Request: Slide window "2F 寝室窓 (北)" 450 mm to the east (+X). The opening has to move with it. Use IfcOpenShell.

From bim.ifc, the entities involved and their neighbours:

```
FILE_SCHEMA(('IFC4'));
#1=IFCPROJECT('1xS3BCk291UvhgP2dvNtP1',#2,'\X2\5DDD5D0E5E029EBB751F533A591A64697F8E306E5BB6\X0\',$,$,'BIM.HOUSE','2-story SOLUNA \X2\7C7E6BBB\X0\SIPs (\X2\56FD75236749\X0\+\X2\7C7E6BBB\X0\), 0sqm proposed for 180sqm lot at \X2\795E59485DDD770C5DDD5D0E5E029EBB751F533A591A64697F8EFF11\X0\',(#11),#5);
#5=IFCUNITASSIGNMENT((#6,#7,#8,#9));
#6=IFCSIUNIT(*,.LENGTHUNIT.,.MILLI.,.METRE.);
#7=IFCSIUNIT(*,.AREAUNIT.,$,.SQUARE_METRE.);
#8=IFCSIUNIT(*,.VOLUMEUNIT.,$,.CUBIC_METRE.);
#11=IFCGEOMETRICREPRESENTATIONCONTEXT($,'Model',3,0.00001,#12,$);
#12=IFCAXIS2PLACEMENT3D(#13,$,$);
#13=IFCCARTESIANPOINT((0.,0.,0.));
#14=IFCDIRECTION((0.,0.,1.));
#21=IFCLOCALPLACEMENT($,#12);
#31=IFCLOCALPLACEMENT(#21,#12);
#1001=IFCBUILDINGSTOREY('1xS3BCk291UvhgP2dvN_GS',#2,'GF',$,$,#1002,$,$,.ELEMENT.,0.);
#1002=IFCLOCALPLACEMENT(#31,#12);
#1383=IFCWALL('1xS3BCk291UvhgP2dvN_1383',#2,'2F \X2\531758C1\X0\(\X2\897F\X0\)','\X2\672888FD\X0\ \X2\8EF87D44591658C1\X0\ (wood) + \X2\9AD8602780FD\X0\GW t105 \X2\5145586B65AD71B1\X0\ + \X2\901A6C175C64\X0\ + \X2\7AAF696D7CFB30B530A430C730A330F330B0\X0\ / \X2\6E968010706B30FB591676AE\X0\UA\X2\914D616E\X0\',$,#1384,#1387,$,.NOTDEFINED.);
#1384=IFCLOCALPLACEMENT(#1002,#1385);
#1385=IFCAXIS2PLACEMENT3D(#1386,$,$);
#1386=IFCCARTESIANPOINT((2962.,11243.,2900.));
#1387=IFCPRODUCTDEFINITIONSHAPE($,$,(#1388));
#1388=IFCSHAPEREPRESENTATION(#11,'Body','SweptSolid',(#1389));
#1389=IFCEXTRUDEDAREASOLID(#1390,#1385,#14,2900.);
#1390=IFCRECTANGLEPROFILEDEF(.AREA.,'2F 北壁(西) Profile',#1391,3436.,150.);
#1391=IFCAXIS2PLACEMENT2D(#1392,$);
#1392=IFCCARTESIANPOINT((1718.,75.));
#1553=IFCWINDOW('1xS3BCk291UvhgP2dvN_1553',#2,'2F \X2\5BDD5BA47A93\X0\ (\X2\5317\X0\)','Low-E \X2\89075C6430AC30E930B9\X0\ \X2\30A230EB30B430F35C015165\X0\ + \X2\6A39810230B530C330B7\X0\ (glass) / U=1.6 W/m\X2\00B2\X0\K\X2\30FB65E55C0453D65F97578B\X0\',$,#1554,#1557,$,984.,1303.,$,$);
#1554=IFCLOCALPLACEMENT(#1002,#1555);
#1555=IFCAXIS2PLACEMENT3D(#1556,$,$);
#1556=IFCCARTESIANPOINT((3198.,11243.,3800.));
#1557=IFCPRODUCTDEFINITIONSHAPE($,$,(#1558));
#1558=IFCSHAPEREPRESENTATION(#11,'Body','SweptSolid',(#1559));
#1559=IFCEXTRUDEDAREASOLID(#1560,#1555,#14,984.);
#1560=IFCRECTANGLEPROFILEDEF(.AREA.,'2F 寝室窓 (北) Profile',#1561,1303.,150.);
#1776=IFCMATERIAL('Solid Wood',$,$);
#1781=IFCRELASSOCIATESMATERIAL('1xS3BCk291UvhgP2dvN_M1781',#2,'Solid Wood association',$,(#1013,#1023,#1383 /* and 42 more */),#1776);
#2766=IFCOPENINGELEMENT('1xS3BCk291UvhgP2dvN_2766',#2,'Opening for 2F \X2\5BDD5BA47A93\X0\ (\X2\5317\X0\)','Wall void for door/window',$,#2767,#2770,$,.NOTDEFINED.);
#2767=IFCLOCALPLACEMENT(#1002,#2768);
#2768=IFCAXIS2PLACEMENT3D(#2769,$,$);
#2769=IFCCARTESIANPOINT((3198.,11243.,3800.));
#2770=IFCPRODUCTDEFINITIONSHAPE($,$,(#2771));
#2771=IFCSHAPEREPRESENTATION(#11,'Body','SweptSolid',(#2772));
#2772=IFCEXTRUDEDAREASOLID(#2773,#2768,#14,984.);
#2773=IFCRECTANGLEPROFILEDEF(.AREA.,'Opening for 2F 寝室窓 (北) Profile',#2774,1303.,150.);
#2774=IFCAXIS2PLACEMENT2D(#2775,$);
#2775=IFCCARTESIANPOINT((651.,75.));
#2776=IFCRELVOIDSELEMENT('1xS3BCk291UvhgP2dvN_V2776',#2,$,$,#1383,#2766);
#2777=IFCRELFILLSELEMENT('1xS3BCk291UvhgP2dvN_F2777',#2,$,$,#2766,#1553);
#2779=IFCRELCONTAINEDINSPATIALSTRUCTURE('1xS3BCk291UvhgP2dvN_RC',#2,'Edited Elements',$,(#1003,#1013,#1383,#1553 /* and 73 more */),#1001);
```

```python
import ifcopenshell
import ifcopenshell.api.geometry
import ifcopenshell.util.placement
import ifcopenshell.util.unit

model = ifcopenshell.open("bim.ifc")
unit_scale = ifcopenshell.util.unit.calculate_unit_scale(model)

window = model.by_guid("1xS3BCk291UvhgP2dvN_1553")
opening = window.FillsVoids[0].RelatingOpeningElement
wall = opening.VoidsElements[0].RelatingBuildingElement

wall_matrix = ifcopenshell.util.placement.get_local_placement(wall.ObjectPlacement)
shift = wall_matrix[:3, 0] * 0.45 / unit_scale
before = ifcopenshell.util.placement.get_local_placement(window.ObjectPlacement)[:3, 3].copy()

# The window is not placed relative to its opening, so move both.
for product in (opening, window):
    matrix = ifcopenshell.util.placement.get_local_placement(product.ObjectPlacement)
    matrix[:3, 3] += shift
    ifcopenshell.api.geometry.edit_object_placement(model, product=product, matrix=matrix, is_si=False)

after = ifcopenshell.util.placement.get_local_placement(window.ObjectPlacement)[:3, 3]
print("window moved by", (after - before).round(3) + 0.0)

model.write("bim_edited.ifc")
```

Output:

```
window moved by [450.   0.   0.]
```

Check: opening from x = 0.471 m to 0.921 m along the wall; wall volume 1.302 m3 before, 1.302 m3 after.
